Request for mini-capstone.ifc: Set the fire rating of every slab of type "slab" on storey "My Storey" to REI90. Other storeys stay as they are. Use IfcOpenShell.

First a look at what the model holds.

```python
import ifcopenshell
import ifcopenshell.util.element

model = ifcopenshell.open("mini-capstone.ifc")
print(model.schema)
storey = next(s for s in model.by_type("IfcBuildingStorey") if s.Name == "My Storey")
slabs = [e for e in ifcopenshell.util.element.get_decomposition(storey) if e.is_a("IfcSlab")]
seen = {}
for e in slabs:
    element_type = ifcopenshell.util.element.get_type(e)
    key = (element_type.Name if element_type != e and element_type else None, ifcopenshell.util.element.get_pset(e, "Pset_SlabCommon", "FireRating"))
    seen[key] = seen.get(key, 0) + 1
for (name, value), count in sorted(seen.items(), key=str):
    print(count, "x", name, "|", value)
```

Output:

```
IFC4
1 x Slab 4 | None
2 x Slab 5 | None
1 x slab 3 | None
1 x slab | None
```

```python
import ifcopenshell
import ifcopenshell.api.pset
import ifcopenshell.util.element

model = ifcopenshell.open("mini-capstone.ifc")

storey = next(s for s in model.by_type("IfcBuildingStorey") if s.Name == "My Storey")
slabs = [e for e in ifcopenshell.util.element.get_decomposition(storey) if e.is_a("IfcSlab")]

count = 0
for e in slabs:
    element_type = ifcopenshell.util.element.get_type(e)
    if element_type in (None, e) or element_type.Name != "slab":
        continue
    # add_pset returns the element's existing set when there is one.
    pset = ifcopenshell.api.pset.add_pset(model, product=e, name="Pset_SlabCommon")
    ifcopenshell.api.pset.edit_pset(model, pset=pset, properties={"FireRating": "REI90"})
    count += 1

print(count, "slabs updated")

model.write("mini-capstone_rev.ifc")
```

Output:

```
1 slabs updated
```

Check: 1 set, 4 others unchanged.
